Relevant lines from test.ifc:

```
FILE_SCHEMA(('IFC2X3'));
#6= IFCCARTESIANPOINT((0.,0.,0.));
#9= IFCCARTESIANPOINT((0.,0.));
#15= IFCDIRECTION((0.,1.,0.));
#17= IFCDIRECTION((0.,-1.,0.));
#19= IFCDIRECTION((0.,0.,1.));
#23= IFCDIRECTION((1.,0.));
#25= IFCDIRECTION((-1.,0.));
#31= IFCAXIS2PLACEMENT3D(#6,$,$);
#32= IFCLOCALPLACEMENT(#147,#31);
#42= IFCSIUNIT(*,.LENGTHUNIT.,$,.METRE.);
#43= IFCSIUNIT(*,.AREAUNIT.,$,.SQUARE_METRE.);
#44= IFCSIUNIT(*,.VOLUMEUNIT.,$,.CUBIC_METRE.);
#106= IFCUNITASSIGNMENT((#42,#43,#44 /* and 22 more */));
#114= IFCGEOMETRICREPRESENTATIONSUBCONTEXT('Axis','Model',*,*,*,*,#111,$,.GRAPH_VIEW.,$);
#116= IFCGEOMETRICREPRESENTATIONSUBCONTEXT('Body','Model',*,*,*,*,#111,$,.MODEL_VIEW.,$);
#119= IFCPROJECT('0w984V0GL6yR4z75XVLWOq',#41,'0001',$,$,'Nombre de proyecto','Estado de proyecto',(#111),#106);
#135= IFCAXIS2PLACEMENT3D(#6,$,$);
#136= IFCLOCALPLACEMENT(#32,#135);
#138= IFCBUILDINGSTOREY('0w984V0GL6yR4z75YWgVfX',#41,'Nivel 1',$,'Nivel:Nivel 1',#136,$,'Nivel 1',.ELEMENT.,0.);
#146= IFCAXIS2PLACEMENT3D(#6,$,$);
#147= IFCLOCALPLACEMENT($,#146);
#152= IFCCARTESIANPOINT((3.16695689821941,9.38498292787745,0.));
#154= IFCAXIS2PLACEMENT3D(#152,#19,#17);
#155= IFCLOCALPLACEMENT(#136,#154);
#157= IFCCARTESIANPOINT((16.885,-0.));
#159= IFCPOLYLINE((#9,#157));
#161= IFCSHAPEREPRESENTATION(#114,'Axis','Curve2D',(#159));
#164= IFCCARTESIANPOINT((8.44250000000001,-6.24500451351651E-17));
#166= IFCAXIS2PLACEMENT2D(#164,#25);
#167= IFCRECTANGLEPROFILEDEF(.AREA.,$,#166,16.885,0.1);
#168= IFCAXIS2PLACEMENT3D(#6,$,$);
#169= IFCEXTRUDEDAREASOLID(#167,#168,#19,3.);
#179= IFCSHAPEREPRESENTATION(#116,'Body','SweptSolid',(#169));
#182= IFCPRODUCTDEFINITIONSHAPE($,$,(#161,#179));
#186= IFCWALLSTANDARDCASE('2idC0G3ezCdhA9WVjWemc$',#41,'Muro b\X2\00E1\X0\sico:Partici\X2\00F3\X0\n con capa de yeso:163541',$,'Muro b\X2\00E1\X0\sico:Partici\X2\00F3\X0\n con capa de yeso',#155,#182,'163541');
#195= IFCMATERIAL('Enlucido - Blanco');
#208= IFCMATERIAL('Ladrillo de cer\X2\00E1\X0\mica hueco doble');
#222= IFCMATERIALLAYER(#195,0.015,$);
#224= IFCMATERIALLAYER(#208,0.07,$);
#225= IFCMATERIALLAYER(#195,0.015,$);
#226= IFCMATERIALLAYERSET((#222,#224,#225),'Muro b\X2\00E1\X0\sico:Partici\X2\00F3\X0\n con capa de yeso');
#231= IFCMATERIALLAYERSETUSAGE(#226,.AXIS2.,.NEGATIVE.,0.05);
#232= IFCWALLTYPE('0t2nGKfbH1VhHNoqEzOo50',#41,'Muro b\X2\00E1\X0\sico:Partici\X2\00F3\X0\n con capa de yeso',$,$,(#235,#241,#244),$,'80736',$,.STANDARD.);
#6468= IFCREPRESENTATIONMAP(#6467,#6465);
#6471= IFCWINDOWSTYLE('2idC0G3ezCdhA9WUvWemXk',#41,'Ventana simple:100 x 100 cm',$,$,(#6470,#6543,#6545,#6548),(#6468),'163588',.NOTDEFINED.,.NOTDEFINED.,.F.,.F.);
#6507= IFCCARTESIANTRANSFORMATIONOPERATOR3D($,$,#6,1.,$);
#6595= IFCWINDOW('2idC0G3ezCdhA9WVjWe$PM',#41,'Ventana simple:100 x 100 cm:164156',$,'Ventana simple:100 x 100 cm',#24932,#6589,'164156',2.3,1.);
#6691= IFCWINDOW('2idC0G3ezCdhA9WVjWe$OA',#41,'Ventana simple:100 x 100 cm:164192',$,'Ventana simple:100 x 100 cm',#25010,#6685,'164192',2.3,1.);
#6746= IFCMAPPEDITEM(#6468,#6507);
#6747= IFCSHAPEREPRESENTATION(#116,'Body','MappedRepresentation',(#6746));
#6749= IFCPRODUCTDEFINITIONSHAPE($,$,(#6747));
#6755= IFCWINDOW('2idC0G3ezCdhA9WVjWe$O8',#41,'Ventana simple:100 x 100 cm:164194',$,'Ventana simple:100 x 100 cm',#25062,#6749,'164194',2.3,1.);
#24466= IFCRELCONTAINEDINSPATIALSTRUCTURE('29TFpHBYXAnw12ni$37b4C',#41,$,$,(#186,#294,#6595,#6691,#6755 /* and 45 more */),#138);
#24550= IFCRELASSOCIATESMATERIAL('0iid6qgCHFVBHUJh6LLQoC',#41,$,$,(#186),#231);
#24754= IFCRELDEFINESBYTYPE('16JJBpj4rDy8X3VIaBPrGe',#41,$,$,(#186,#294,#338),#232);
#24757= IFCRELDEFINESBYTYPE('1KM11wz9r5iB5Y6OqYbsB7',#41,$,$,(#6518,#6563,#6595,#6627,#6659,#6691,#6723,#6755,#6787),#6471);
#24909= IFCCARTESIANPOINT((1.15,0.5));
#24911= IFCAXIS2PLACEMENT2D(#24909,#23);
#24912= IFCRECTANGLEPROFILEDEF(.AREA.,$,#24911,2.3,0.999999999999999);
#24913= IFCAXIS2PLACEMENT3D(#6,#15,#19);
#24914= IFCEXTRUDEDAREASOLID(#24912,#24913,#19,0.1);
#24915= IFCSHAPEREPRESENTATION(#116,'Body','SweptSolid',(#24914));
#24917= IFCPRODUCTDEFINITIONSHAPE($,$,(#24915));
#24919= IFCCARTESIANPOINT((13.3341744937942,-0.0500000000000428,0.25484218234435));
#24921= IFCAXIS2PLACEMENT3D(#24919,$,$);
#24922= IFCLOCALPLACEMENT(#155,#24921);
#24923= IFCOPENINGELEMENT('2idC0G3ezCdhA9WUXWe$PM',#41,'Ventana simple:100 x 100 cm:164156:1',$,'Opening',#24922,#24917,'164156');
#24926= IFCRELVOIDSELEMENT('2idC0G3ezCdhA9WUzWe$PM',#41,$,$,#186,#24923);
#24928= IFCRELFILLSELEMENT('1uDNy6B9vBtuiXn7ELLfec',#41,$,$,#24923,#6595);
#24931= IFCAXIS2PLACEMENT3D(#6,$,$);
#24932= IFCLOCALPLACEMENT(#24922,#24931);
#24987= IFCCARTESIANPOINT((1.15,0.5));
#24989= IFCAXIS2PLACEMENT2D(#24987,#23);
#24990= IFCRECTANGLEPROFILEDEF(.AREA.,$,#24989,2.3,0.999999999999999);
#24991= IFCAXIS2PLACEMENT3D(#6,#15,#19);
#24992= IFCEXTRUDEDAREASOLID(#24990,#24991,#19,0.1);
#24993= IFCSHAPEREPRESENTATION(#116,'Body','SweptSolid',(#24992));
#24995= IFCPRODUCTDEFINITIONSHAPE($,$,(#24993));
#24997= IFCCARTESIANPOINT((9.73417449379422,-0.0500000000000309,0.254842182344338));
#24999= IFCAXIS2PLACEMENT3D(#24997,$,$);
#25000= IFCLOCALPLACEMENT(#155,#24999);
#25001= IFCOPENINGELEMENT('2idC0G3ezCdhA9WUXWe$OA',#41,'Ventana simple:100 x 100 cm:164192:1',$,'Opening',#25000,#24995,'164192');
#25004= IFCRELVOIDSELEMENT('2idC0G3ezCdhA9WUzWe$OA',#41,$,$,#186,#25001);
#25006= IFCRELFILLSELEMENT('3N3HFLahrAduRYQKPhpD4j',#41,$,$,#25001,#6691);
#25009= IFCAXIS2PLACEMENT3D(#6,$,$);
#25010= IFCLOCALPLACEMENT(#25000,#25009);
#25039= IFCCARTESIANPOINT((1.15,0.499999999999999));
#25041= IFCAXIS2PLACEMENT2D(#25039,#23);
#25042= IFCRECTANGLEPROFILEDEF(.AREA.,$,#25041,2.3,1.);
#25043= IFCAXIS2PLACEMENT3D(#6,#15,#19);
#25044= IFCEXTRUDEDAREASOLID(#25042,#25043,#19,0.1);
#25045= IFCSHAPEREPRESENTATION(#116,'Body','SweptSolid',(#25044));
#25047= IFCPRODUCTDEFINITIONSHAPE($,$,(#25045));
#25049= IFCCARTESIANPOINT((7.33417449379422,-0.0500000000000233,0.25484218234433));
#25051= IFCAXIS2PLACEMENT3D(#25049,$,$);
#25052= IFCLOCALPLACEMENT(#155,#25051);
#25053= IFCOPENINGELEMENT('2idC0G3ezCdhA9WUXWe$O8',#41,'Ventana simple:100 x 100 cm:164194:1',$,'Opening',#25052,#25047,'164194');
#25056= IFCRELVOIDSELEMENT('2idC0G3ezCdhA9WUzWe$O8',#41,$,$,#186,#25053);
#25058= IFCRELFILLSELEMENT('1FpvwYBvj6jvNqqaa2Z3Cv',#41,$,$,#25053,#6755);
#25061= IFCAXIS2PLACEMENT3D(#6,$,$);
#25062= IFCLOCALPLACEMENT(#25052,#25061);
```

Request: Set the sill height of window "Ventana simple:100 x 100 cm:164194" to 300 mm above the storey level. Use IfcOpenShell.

```python
import numpy as np
import ifcopenshell
import ifcopenshell.api.geometry
import ifcopenshell.geom
import ifcopenshell.util.element
import ifcopenshell.util.placement
import ifcopenshell.util.shape
import ifcopenshell.util.unit

model = ifcopenshell.open("test.ifc")
unit_scale = ifcopenshell.util.unit.calculate_unit_scale(model)

window = model.by_guid("2idC0G3ezCdhA9WVjWe$O8")
opening = window.FillsVoids[0].RelatingOpeningElement
storey = ifcopenshell.util.element.get_container(window, ifc_class="IfcBuildingStorey")
level = ifcopenshell.util.placement.get_local_placement(storey.ObjectPlacement)[2, 3]

# The opening's origin need not be at the sill, so measure its lowest point.
shape = ifcopenshell.geom.create_shape(ifcopenshell.geom.settings(), opening)
bottom = ifcopenshell.util.shape.get_shape_bottom_elevation(shape, shape.geometry) / unit_scale
dz = level + 0.3 / unit_scale - bottom

shift = np.array([0.0, 0.0, dz])
# The window is placed relative to its opening, so it follows when the opening moves.
matrix = ifcopenshell.util.placement.get_local_placement(opening.ObjectPlacement)
matrix[:3, 3] += shift
ifcopenshell.api.geometry.edit_object_placement(
    model, product=opening, matrix=matrix, is_si=False, should_transform_children=True
)

print(f"moved by {dz * unit_scale:+.3f} m")

model.write("test-out.ifc")
```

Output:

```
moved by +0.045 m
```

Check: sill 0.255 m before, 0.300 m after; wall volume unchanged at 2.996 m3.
